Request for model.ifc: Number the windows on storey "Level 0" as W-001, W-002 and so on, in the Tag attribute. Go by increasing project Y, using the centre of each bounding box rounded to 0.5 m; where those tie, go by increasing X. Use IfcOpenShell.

First a look at what the model holds.

```python
import ifcopenshell
import ifcopenshell.util.element
import ifcopenshell.util.placement

model = ifcopenshell.open("model.ifc")
print(model.schema)
storey = next(s for s in model.by_type("IfcBuildingStorey") if s.Name == "Level 0")
windows = [e for e in ifcopenshell.util.element.get_decomposition(storey) if e.is_a("IfcWindow")]
for e in sorted(windows, key=lambda e: e.id()):
    origin = ifcopenshell.util.placement.get_local_placement(e.ObjectPlacement)[:3, 3]
    print(e.id(), e.Tag, e.Name, origin.round(2) + 0.0, sep=" | ")
```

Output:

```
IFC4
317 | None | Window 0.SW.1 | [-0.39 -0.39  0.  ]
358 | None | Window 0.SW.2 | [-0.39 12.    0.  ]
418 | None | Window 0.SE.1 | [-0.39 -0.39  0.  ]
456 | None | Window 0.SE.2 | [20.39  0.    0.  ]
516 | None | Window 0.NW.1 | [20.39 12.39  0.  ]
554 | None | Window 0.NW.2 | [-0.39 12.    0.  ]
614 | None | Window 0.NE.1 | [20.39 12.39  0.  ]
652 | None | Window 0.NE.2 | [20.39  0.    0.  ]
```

```python
import ifcopenshell
import ifcopenshell.geom
import ifcopenshell.util.element
import ifcopenshell.util.shape

model = ifcopenshell.open("model.ifc")
settings = ifcopenshell.geom.settings()
settings.set("use-world-coords", True)


def centre(element):
    shape = ifcopenshell.geom.create_shape(settings, element)
    return ifcopenshell.util.shape.get_bbox_centroid(shape.geometry)


storey = next(s for s in model.by_type("IfcBuildingStorey") if s.Name == "Level 0")
windows = [e for e in ifcopenshell.util.element.get_decomposition(storey) if e.is_a("IfcWindow")]

# Insertion points can sit at a corner or the storey origin, so sort by the geometry (in metres).
centres = {e: centre(e) for e in windows}
windows.sort(key=lambda e: (round(centres[e][1] / 0.5), centres[e][0]))

for i, e in enumerate(windows, start=1):
    number = f"W-0{i:02d}"
    e.Tag = number
    print(e.id(), number)

model.write("model_rev.ifc")
```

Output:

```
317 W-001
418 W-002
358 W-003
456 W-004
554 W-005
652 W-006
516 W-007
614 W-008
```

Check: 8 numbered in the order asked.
